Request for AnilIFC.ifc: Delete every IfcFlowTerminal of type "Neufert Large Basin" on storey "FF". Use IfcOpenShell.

First a look at what the model holds.

```python
import ifcopenshell
import ifcopenshell.util.element

model = ifcopenshell.open("AnilIFC.ifc")
print(model.schema)
storey = next(s for s in model.by_type("IfcBuildingStorey") if s.Name == "FF")
terminals = [e for e in ifcopenshell.util.element.get_decomposition(storey) if e.is_a("IfcFlowTerminal")]
seen = {}
for e in terminals:
    element_type = ifcopenshell.util.element.get_type(e)
    name = element_type.Name if element_type not in (None, e) else None
    seen[name] = seen.get(name, 0) + 1
for name, count in sorted(seen.items(), key=str):
    print(count, "x", name)
```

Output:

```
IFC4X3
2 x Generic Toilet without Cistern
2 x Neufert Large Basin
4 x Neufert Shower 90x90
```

```python
import ifcopenshell
import ifcopenshell.api.root
import ifcopenshell.util.element

model = ifcopenshell.open("AnilIFC.ifc")

storey = next(s for s in model.by_type("IfcBuildingStorey") if s.Name == "FF")
terminals = [e for e in ifcopenshell.util.element.get_decomposition(storey) if e.is_a("IfcFlowTerminal")]
targets = [e for e in terminals if (t := ifcopenshell.util.element.get_type(e)) not in (None, e) and t.Name == "Neufert Large Basin"]

for e in targets:
    ifcopenshell.api.root.remove_product(model, product=e)
print(len(targets), "removed")

model.write("AnilIFC_updated.ifc")
```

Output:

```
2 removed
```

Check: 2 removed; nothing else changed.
